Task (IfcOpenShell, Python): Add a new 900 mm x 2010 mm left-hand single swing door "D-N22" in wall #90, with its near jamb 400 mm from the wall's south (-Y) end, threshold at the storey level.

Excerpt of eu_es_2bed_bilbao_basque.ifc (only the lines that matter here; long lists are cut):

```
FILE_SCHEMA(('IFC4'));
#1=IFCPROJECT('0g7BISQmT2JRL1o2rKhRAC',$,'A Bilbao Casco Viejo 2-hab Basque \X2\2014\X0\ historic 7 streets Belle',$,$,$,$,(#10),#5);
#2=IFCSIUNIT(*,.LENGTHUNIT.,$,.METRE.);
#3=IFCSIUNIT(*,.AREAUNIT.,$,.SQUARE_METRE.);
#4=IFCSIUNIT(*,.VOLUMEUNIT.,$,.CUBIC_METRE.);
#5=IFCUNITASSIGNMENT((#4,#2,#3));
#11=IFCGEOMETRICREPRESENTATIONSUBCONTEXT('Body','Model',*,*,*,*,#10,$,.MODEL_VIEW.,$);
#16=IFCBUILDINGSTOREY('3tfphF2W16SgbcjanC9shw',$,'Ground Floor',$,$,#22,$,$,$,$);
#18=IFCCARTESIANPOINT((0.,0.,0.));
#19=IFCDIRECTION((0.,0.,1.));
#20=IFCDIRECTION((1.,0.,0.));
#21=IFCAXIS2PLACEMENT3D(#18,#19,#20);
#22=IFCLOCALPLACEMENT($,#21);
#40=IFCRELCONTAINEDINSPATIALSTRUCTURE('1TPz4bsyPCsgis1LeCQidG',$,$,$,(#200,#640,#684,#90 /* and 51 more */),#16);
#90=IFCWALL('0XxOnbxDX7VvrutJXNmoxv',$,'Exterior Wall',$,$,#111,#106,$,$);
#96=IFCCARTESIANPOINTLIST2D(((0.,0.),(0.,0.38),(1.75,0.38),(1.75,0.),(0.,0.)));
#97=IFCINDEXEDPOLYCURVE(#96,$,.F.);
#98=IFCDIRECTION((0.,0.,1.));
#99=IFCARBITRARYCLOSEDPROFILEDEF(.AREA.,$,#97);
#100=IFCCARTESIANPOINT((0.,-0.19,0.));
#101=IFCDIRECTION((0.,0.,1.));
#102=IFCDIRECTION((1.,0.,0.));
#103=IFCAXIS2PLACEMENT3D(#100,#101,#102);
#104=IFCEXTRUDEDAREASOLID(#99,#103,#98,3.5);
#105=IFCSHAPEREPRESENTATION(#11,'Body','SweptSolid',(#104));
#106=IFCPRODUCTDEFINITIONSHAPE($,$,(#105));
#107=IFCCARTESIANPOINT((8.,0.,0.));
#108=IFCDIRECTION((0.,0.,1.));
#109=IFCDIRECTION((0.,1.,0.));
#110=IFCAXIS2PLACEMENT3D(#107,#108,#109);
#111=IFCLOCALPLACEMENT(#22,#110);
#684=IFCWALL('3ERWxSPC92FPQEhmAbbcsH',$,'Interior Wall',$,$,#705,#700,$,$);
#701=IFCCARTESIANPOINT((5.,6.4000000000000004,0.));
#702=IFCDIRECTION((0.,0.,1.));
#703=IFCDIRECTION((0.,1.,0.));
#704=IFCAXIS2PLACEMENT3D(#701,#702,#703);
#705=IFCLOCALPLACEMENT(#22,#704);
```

```python
import numpy as np
import ifcopenshell
import ifcopenshell.api.feature
import ifcopenshell.api.geometry
import ifcopenshell.api.root
import ifcopenshell.api.spatial
import ifcopenshell.geom
import ifcopenshell.util.element
import ifcopenshell.util.placement
import ifcopenshell.util.representation
import ifcopenshell.util.shape
import ifcopenshell.util.unit

model = ifcopenshell.open("eu_es_2bed_bilbao_basque.ifc")
unit_scale = ifcopenshell.util.unit.calculate_unit_scale(model)
settings = ifcopenshell.geom.settings()


def volume(element):
    """Net volume in cubic metres, openings subtracted."""
    shape = ifcopenshell.geom.create_shape(settings, element)
    return ifcopenshell.util.shape.get_volume(shape.geometry)


wall = model.by_guid("0XxOnbxDX7VvrutJXNmoxv")
storey = ifcopenshell.util.element.get_container(wall, ifc_class="IfcBuildingStorey")
context = ifcopenshell.util.representation.get_context(model, "Model", "Body", "MODEL_VIEW")
before = volume(wall)

width, height, from_end, sill = 0.9, 2.01, 0.4, 0.0  # metres

# The wall runs along its own X axis, and the end named is its -X end.
wall_shape = ifcopenshell.geom.create_shape(settings, wall)
x, y, z = ifcopenshell.util.shape.get_vertices(wall_shape.geometry).T
start = x.min() + from_end
face, thickness = float(y.min()), float(y.max() - y.min())
wall_matrix = ifcopenshell.util.placement.get_local_placement(wall.ObjectPlacement)
level = ifcopenshell.util.placement.get_local_placement(storey.ObjectPlacement)[2, 3]


def in_wall(x, y):
    """Placement at x, y metres in the wall's axes, at sill height."""
    matrix = wall_matrix.copy()
    matrix[:, 3] = wall_matrix @ np.array([x / unit_scale, y / unit_scale, 0.0, 1.0])
    matrix[2, 3] = level + sill / unit_scale
    return matrix


# Opening: a box that overshoots both wall faces by 50 mm.
opening = ifcopenshell.api.root.create_entity(model, ifc_class="IfcOpeningElement", predefined_type="OPENING")
box = ifcopenshell.api.geometry.add_wall_representation(
    model, context=context, length=width, height=height, thickness=thickness + 0.1
)
ifcopenshell.api.geometry.assign_representation(model, product=opening, representation=box)
ifcopenshell.api.geometry.edit_object_placement(model, product=opening, matrix=in_wall(start, face - 0.05), is_si=False)
ifcopenshell.api.feature.add_feature(model, feature=opening, element=wall)

door = ifcopenshell.api.root.create_entity(model, ifc_class="IfcDoor", name="D-N22", predefined_type="DOOR")
door.OverallWidth, door.OverallHeight = width / unit_scale, height / unit_scale
door.OperationType = "SINGLE_SWING_LEFT"
body = ifcopenshell.api.geometry.add_door_representation(
    model,
    context=context,
    overall_width=door.OverallWidth,
    overall_height=door.OverallHeight,
    operation_type="SINGLE_SWING_LEFT",
    lining_properties={"LiningDepth": thickness / unit_scale, "ThresholdDepth": thickness / unit_scale},
)
ifcopenshell.api.geometry.assign_representation(model, product=door, representation=body)
ifcopenshell.api.spatial.assign_container(model, products=[door], relating_structure=storey)
ifcopenshell.api.feature.add_filling(model, opening=opening, element=door)

# The lining spans the wall, so the door starts at the wall face.
ifcopenshell.api.geometry.edit_object_placement(model, product=door, matrix=in_wall(start, face), is_si=False)

after = volume(wall)

print(f"wall volume {before:.3f} -> {after:.3f} m3")

model.write("eu_es_2bed_bilbao_basque_v2.ifc")
```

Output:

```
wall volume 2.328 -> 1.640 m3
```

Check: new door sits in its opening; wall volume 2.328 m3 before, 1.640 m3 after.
